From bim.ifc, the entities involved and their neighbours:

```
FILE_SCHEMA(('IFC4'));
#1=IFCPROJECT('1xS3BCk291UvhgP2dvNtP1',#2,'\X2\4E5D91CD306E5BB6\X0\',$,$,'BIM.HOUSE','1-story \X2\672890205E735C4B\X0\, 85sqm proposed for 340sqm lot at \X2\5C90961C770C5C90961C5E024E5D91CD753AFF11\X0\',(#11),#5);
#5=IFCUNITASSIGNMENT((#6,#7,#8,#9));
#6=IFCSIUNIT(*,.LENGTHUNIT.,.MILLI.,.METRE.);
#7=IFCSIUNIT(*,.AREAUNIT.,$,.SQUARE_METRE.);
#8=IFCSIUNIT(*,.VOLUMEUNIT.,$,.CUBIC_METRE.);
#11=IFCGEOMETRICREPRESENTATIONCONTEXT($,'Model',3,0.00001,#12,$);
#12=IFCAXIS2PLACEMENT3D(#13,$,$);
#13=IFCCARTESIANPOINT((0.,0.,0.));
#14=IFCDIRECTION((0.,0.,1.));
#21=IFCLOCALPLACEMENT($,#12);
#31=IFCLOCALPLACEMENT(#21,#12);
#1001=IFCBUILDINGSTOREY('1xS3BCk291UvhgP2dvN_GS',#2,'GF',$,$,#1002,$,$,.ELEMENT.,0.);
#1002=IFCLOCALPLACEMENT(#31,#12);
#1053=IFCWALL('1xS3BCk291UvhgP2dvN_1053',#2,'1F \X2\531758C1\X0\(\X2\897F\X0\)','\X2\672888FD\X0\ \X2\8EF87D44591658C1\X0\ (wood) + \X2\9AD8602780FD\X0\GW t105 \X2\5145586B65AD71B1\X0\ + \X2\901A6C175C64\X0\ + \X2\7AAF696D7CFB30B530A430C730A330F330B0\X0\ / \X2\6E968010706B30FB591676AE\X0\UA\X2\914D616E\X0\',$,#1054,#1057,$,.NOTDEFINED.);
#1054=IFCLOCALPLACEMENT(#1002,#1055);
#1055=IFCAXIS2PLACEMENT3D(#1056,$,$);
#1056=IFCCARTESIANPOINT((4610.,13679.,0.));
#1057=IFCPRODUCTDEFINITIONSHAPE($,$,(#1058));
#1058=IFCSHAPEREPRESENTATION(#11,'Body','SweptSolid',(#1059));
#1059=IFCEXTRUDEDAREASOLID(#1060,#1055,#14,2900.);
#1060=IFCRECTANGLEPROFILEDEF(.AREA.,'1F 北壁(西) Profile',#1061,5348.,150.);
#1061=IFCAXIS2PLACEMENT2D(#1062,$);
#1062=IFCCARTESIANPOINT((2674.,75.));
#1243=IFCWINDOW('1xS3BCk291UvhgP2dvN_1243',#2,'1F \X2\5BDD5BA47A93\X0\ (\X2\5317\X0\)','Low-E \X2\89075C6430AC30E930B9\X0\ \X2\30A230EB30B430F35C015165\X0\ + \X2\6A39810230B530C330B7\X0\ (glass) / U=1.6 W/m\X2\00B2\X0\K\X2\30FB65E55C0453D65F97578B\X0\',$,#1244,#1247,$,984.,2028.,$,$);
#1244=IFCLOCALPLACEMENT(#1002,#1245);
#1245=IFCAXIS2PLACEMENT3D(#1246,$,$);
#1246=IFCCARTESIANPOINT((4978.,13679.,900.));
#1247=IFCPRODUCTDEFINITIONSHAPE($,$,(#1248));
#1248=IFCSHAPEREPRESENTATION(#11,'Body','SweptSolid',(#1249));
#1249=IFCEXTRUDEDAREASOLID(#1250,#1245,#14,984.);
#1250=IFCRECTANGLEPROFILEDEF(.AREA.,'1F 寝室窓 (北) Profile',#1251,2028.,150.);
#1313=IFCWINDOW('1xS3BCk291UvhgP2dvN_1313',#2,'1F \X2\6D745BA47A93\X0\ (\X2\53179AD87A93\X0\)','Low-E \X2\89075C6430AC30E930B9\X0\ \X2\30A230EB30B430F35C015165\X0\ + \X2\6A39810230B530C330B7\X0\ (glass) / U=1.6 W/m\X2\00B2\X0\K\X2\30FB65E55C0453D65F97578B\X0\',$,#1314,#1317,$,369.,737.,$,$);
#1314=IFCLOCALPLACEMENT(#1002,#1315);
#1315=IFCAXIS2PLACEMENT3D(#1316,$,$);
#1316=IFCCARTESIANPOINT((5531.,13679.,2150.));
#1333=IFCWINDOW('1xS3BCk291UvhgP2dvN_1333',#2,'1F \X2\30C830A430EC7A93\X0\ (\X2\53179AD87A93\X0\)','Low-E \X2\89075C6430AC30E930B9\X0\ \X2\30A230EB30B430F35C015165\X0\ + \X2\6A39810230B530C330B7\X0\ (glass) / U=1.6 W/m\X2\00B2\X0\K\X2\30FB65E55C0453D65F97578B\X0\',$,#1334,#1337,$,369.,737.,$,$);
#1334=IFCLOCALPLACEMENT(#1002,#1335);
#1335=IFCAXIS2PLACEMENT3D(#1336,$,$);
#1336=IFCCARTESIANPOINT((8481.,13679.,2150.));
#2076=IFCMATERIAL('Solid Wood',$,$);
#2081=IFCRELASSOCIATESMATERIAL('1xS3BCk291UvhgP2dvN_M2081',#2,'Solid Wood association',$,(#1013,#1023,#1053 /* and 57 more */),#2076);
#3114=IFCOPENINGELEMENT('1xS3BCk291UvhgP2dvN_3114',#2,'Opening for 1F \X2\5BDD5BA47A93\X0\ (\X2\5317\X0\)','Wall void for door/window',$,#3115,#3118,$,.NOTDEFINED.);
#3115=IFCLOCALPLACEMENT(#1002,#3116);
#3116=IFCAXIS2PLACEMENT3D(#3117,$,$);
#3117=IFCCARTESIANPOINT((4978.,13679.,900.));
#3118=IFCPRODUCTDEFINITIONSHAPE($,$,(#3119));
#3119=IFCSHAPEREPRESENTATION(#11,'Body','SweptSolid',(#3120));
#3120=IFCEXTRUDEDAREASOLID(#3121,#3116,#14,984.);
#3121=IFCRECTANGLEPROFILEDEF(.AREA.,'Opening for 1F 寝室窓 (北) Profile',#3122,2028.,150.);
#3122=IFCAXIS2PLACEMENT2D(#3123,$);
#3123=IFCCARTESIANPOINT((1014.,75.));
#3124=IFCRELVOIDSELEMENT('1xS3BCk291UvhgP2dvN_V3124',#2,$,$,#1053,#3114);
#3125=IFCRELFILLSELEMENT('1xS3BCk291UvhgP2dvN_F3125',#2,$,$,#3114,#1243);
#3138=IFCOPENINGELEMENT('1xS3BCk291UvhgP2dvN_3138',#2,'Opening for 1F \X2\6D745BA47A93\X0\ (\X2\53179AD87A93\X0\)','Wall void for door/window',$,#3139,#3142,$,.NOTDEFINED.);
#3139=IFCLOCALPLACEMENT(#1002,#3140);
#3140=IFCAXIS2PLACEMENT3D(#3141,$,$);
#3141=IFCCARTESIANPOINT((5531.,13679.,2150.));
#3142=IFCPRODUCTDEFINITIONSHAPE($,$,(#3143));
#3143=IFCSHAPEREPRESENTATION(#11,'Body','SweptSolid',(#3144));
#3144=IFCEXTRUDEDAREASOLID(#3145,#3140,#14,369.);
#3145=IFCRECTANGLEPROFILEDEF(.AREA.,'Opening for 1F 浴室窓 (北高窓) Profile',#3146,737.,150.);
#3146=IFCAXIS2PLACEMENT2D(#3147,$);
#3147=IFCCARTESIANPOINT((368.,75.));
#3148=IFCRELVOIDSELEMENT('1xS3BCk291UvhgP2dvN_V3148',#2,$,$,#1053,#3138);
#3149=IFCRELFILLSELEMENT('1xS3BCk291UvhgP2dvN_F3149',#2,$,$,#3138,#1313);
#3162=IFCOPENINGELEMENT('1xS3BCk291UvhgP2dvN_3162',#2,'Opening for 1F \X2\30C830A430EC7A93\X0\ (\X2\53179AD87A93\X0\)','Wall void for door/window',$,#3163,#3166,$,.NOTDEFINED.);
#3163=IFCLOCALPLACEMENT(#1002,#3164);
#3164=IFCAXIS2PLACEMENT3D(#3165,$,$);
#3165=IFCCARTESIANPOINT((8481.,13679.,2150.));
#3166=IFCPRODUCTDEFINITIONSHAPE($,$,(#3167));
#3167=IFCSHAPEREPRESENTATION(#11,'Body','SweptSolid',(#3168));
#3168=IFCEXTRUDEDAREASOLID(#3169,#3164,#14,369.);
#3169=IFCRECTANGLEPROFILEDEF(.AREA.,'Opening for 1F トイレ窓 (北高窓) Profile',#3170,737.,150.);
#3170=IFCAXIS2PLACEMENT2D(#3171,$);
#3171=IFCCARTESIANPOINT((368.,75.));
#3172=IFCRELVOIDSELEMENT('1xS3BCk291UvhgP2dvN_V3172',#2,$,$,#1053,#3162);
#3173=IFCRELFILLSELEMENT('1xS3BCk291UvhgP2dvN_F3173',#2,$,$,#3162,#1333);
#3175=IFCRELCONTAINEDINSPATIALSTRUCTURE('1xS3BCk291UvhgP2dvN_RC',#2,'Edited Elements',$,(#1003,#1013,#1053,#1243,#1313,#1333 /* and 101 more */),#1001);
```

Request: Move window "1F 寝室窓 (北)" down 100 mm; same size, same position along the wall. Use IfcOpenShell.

```python
import numpy as np
import ifcopenshell
import ifcopenshell.api.geometry
import ifcopenshell.util.placement
import ifcopenshell.util.unit

model = ifcopenshell.open("bim.ifc")
unit_scale = ifcopenshell.util.unit.calculate_unit_scale(model)

window = model.by_guid("1xS3BCk291UvhgP2dvN_1243")
opening = window.FillsVoids[0].RelatingOpeningElement
dz = -0.1 / unit_scale

shift = np.array([0.0, 0.0, dz])
# The window is not placed relative to its opening, so move both.
for product in (opening, window):
    matrix = ifcopenshell.util.placement.get_local_placement(product.ObjectPlacement)
    matrix[:3, 3] += shift
    ifcopenshell.api.geometry.edit_object_placement(model, product=product, matrix=matrix, is_si=False)

print(f"moved by {dz * unit_scale:+.3f} m")

model.write("bim_rev.ifc")
```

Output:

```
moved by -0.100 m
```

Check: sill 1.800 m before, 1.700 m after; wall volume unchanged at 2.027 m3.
